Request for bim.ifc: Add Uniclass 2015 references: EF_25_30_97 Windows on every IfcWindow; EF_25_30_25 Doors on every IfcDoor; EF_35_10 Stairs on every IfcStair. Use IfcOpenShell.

First a look at what the model holds.

```python
import ifcopenshell

model = ifcopenshell.open("bim.ifc")
print(model.schema)
print("classifications:", [c.Name for c in model.by_type("IfcClassification")])
for ifc_class in ("IfcDoor", "IfcRoof", "IfcStair", "IfcWall", "IfcWindow"):
    print(ifc_class, len(model.by_type(ifc_class)))
```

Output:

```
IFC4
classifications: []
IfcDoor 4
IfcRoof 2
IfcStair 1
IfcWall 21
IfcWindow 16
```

```python
import ifcopenshell
import ifcopenshell.api.classification

model = ifcopenshell.open("bim.ifc")

system = ifcopenshell.api.classification.add_classification(model, classification="Uniclass 2015")

codes = {
    "IfcWindow": ("EF_25_30_97", "Windows"),
    "IfcDoor": ("EF_25_30_25", "Doors"),
    "IfcStair": ("EF_35_10", "Stairs"),
}
for ifc_class, (code, name) in codes.items():
    products = model.by_type(ifc_class)
    ifcopenshell.api.classification.add_reference(
        model, products=products, classification=system, identification=code, name=name
    )
    print(code, len(products))

model.write("bim_updated.ifc")
```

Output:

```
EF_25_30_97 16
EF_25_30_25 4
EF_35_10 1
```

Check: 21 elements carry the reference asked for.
